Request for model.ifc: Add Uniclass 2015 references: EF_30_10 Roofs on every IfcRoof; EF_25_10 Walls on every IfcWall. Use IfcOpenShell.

First a look at what the model holds.

```python
import ifcopenshell

model = ifcopenshell.open("model.ifc")
print(model.schema)
print("classifications:", [c.Name for c in model.by_type("IfcClassification")])
for ifc_class in ("IfcDoor", "IfcRoof", "IfcStair", "IfcWall", "IfcWindow"):
    print(ifc_class, len(model.by_type(ifc_class)))
```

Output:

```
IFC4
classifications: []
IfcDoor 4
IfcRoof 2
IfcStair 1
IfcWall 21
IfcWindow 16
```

```python
import ifcopenshell
import ifcopenshell.api.classification

model = ifcopenshell.open("model.ifc")

system = ifcopenshell.api.classification.add_classification(model, classification="Uniclass 2015")

codes = {
    "IfcRoof": ("EF_30_10", "Roofs"),
    "IfcWall": ("EF_25_10", "Walls"),
}
for ifc_class, (code, name) in codes.items():
    products = model.by_type(ifc_class)
    ifcopenshell.api.classification.add_reference(
        model, products=products, classification=system, identification=code, name=name
    )
    print(code, len(products))

model.write("model_edited.ifc")
```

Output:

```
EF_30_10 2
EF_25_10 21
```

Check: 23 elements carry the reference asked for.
